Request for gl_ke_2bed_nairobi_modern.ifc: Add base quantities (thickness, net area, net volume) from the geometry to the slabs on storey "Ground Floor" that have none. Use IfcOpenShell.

First a look at what the model holds.

```python
import ifcopenshell
import ifcopenshell.util.element
import ifcopenshell.util.unit

model = ifcopenshell.open("gl_ke_2bed_nairobi_modern.ifc")
print(model.schema)
for unit_type in ("LENGTHUNIT", "AREAUNIT", "VOLUMEUNIT"):
    print(unit_type, ifcopenshell.util.unit.calculate_unit_scale(model, unit_type))
storey = next(s for s in model.by_type("IfcBuildingStorey") if s.Name == "Ground Floor")
slabs = [e for e in ifcopenshell.util.element.get_decomposition(storey) if e.is_a("IfcSlab")]
for e in sorted(slabs, key=lambda e: e.id()):
    print(e.id(), e.is_a(), e.Name, list(ifcopenshell.util.element.get_psets(e, qtos_only=True)), sep=" | ")
```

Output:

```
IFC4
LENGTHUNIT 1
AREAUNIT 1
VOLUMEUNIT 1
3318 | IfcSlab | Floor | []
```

```python
import ifcopenshell
import ifcopenshell.api.pset
import ifcopenshell.geom
import ifcopenshell.util.element
import ifcopenshell.util.shape
import ifcopenshell.util.unit

model = ifcopenshell.open("gl_ke_2bed_nairobi_modern.ifc")
unit_scale = ifcopenshell.util.unit.calculate_unit_scale(model)
area_scale = ifcopenshell.util.unit.calculate_unit_scale(model, "AREAUNIT")
volume_scale = ifcopenshell.util.unit.calculate_unit_scale(model, "VOLUMEUNIT")
settings = ifcopenshell.geom.settings()

storey = next(s for s in model.by_type("IfcBuildingStorey") if s.Name == "Ground Floor")
slabs = [e for e in ifcopenshell.util.element.get_decomposition(storey) if e.is_a("IfcSlab")]

for e in sorted(slabs, key=lambda e: e.id()):
    if ifcopenshell.util.element.get_psets(e, qtos_only=True, should_inherit=False):
        continue
    # Geometry comes back in metres, in the element's own axes.
    shape = ifcopenshell.geom.create_shape(settings, e)
    values = {
        "Width": ifcopenshell.util.shape.get_z(shape.geometry) / unit_scale,
        "NetArea": ifcopenshell.util.shape.get_footprint_area(shape.geometry) / area_scale,
        "NetVolume": ifcopenshell.util.shape.get_volume(shape.geometry) / volume_scale,
    }
    qto = ifcopenshell.api.pset.add_qto(model, product=e, name="Qto_SlabBaseQuantities")
    ifcopenshell.api.pset.edit_qto(model, qto=qto, properties=values)
    print(e.id(), {k: round(v, 3) for k, v in values.items()})

model.write("gl_ke_2bed_nairobi_modern-out.ifc")
```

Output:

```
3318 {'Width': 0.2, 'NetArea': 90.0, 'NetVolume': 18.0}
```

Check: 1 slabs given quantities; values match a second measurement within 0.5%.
